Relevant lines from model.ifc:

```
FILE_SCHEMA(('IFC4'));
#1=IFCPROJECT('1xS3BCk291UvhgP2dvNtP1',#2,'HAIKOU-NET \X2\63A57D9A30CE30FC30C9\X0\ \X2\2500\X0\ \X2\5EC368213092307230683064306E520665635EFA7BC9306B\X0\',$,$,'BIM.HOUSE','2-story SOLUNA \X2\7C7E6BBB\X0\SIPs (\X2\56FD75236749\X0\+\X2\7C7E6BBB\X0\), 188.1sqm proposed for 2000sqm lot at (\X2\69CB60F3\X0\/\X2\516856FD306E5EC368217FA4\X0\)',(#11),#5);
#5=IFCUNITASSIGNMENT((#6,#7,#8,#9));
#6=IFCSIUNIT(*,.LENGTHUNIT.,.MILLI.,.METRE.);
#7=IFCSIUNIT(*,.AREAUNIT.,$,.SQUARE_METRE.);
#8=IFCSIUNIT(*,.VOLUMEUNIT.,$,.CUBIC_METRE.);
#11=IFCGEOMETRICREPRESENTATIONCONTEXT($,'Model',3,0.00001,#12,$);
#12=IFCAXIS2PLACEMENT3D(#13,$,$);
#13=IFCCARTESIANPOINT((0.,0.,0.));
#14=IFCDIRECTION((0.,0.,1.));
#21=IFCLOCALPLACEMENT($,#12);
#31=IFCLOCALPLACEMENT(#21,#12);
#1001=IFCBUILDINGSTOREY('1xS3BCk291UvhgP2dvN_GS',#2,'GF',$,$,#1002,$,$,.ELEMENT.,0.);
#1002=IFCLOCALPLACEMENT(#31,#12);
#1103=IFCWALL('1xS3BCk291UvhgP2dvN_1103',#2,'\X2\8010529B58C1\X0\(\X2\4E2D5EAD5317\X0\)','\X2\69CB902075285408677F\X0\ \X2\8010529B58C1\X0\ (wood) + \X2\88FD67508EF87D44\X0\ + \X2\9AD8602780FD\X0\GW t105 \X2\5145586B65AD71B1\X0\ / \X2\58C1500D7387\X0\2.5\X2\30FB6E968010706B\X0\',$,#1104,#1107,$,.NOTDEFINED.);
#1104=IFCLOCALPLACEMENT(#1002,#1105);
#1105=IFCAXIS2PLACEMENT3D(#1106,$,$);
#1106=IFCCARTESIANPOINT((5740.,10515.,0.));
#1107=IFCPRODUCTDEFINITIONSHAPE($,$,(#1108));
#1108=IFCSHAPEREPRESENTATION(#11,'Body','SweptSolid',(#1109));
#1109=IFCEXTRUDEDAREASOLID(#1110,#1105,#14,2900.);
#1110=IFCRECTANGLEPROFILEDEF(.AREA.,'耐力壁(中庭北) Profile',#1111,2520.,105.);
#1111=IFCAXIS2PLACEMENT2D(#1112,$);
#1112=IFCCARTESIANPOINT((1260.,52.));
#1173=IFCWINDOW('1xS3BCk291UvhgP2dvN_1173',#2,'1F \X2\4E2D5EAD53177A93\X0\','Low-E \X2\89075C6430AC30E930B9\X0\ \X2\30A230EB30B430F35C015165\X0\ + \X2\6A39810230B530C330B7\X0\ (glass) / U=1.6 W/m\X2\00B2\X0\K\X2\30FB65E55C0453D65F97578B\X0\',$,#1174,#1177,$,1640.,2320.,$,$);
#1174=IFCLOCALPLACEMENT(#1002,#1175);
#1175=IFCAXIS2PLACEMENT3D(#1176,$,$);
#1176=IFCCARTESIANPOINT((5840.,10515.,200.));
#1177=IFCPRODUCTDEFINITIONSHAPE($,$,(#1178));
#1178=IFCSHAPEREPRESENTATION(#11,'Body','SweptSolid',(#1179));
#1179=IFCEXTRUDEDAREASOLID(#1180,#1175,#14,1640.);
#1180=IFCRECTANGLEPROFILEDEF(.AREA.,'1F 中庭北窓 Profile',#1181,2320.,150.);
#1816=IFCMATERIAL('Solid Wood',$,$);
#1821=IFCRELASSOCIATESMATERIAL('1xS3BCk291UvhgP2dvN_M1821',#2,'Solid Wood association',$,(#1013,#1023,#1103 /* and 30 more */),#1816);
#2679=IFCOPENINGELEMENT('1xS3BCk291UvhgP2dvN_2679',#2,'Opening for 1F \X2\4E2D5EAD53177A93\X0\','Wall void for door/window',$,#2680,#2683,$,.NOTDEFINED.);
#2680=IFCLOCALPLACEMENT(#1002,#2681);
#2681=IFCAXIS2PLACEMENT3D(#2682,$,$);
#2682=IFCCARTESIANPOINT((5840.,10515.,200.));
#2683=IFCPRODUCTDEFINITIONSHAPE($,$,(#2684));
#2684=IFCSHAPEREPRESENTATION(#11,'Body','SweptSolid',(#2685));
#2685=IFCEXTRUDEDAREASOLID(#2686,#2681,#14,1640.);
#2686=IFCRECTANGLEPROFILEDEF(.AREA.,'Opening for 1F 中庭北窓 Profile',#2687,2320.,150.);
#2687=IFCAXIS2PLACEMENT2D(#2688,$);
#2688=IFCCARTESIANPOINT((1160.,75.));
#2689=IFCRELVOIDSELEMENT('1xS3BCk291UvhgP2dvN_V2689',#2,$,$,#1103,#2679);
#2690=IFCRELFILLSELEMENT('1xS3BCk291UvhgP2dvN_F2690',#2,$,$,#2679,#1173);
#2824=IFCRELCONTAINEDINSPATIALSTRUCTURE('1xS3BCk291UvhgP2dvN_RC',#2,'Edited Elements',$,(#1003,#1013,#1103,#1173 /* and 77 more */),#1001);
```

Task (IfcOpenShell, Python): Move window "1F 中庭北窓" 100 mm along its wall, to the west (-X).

```python
import ifcopenshell
import ifcopenshell.api.geometry
import ifcopenshell.util.placement

model = ifcopenshell.open("model.ifc")

window = model.by_id(1173)
opening = window.FillsVoids[0].RelatingOpeningElement
wall = opening.VoidsElements[0].RelatingBuildingElement

wall_matrix = ifcopenshell.util.placement.get_local_placement(wall.ObjectPlacement)
shift = wall_matrix[:3, 0] * -100.0
before = ifcopenshell.util.placement.get_local_placement(window.ObjectPlacement)[:3, 3].copy()

# The window is not placed relative to its opening, so move both.
for product in (opening, window):
    matrix = ifcopenshell.util.placement.get_local_placement(product.ObjectPlacement)
    matrix[:3, 3] += shift
    ifcopenshell.api.geometry.edit_object_placement(model, product=product, matrix=matrix, is_si=False)

after = ifcopenshell.util.placement.get_local_placement(window.ObjectPlacement)[:3, 3]
print("window moved by", (after - before).round(3) + 0.0)

model.write("model_rev.ifc")
```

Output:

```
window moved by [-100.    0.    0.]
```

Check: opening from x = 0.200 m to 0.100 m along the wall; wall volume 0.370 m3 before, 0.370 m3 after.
